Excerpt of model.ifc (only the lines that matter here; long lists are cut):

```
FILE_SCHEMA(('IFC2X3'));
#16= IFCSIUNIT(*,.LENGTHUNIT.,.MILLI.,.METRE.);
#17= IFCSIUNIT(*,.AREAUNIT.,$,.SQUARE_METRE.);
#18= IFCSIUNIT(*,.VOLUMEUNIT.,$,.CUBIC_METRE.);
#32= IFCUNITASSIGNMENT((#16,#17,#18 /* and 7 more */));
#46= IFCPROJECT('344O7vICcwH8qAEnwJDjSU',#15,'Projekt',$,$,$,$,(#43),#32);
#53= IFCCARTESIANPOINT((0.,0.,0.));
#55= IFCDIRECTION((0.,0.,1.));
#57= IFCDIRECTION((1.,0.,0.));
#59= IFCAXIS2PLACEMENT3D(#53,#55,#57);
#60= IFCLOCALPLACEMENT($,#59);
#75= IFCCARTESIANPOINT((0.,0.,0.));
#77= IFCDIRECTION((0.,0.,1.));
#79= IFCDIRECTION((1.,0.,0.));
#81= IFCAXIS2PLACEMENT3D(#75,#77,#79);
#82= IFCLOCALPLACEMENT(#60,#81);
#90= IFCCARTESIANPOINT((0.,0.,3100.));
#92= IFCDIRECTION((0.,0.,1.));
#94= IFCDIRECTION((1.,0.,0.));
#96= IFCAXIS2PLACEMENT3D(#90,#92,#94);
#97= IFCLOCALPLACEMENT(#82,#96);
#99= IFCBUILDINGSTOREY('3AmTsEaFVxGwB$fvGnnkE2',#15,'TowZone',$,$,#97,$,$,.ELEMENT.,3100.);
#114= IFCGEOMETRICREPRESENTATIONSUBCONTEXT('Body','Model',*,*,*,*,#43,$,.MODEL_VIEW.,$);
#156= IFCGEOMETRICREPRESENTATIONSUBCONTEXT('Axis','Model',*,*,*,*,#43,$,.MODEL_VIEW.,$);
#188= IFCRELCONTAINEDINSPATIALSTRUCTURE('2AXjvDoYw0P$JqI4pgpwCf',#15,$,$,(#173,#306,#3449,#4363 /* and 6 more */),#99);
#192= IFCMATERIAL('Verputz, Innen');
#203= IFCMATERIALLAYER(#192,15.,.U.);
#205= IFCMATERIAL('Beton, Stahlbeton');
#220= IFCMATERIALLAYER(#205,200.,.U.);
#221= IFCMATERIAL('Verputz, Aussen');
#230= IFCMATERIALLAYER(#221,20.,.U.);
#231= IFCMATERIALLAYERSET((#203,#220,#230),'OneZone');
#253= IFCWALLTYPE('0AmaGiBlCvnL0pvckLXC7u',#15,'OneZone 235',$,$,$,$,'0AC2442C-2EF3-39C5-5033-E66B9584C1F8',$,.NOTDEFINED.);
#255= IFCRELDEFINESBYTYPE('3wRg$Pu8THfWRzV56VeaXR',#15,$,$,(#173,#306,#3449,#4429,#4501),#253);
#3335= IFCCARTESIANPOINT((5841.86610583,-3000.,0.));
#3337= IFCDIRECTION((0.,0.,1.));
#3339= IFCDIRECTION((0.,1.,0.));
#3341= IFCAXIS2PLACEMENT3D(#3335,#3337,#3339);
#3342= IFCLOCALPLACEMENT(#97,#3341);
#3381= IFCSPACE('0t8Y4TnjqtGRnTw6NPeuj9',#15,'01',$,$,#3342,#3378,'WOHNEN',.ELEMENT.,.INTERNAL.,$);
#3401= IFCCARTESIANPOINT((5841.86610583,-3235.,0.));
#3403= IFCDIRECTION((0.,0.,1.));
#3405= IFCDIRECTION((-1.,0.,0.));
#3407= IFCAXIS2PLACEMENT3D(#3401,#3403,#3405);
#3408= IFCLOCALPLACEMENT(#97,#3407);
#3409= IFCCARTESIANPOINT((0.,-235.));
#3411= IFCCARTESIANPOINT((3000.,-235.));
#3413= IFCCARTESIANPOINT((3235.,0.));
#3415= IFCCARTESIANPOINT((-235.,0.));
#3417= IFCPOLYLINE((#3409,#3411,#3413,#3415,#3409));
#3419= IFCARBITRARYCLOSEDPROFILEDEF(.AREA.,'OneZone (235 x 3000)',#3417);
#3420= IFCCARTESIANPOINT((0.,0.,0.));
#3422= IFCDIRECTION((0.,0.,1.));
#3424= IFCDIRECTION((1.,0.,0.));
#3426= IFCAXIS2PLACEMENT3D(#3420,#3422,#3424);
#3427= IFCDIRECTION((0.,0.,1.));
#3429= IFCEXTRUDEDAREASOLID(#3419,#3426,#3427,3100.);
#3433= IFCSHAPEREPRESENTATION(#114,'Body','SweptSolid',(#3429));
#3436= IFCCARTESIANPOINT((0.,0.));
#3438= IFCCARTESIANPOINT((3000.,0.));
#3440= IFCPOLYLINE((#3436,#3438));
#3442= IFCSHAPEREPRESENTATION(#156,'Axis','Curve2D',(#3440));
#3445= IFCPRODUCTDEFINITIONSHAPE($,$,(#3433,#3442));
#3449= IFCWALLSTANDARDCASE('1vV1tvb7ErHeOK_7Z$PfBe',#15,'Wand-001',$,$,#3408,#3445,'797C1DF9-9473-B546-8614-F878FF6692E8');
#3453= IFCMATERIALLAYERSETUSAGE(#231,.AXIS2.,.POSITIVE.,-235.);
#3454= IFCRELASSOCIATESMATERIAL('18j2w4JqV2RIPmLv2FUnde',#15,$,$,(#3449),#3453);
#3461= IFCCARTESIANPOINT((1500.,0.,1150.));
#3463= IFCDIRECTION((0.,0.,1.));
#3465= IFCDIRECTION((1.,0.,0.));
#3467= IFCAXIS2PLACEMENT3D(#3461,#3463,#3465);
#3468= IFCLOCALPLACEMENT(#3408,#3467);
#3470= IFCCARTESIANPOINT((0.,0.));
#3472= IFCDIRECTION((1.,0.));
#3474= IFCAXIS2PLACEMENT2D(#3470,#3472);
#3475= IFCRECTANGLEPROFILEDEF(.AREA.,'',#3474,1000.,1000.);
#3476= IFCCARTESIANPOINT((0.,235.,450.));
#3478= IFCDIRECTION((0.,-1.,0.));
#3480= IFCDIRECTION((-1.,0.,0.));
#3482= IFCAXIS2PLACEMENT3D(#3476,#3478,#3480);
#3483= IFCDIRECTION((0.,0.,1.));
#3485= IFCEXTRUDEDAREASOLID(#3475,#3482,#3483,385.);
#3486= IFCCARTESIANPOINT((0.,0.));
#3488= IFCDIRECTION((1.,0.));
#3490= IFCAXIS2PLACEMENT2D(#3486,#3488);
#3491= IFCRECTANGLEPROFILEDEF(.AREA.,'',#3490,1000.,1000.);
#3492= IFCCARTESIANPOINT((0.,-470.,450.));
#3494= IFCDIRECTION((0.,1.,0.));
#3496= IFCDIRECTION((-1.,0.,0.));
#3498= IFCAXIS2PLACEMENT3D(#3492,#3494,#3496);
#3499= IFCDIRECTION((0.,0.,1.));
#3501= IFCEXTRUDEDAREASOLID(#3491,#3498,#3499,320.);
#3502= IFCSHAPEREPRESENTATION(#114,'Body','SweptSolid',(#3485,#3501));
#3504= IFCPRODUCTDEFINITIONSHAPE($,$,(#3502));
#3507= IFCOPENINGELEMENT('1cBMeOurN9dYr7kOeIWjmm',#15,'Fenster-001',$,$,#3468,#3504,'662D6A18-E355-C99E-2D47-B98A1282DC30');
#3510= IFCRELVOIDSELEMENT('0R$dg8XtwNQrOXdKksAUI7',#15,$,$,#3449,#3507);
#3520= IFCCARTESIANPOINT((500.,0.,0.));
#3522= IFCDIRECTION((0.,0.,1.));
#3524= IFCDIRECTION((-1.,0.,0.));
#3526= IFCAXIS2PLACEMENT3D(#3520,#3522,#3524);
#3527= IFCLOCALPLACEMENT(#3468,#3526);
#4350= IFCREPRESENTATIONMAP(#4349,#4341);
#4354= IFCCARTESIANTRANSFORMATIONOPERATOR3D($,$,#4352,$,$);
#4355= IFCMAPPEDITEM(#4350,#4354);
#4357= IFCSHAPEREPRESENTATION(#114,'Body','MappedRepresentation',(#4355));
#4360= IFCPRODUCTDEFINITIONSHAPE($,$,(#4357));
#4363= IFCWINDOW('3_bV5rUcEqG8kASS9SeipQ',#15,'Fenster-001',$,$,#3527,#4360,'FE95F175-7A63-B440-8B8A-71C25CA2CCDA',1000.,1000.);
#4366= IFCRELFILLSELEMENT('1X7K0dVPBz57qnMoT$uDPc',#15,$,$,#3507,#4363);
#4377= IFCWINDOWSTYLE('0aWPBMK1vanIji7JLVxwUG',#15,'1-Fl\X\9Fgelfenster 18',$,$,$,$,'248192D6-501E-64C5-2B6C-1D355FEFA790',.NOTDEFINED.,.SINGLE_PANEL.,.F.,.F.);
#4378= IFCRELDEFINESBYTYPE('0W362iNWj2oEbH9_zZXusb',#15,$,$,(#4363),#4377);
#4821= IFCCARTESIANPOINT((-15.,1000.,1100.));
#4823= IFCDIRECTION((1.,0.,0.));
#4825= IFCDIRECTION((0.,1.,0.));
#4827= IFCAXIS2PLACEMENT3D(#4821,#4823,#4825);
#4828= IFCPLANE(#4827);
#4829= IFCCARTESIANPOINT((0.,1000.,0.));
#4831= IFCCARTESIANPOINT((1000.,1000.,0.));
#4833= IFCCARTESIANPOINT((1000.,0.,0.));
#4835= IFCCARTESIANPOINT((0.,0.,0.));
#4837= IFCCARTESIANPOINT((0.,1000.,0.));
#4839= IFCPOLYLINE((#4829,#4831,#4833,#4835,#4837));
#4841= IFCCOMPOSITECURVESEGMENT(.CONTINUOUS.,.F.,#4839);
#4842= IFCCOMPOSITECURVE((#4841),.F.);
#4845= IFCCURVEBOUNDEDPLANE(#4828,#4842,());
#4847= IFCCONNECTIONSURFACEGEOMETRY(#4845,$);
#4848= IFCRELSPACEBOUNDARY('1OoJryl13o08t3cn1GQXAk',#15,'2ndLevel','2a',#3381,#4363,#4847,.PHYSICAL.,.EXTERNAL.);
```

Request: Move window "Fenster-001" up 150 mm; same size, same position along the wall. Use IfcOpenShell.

```python
import numpy as np
import ifcopenshell
import ifcopenshell.api.geometry
import ifcopenshell.util.placement
import ifcopenshell.util.unit

model = ifcopenshell.open("model.ifc")
unit_scale = ifcopenshell.util.unit.calculate_unit_scale(model)

window = model.by_id(4363)
opening = window.FillsVoids[0].RelatingOpeningElement
dz = 150.0

shift = np.array([0.0, 0.0, dz])
# The window is placed relative to its opening, so it follows when the opening moves.
matrix = ifcopenshell.util.placement.get_local_placement(opening.ObjectPlacement)
matrix[:3, 3] += shift
ifcopenshell.api.geometry.edit_object_placement(
    model, product=opening, matrix=matrix, is_si=False, should_transform_children=True
)

# Space boundary surfaces are stored in each space's coordinates; move them too.
for rel in window.ProvidesBoundaries:
    if not rel.ConnectionGeometry:
        continue
    surface = rel.ConnectionGeometry.SurfaceOnRelatingElement.BasisSurface
    space_matrix = ifcopenshell.util.placement.get_local_placement(rel.RelatingSpace.ObjectPlacement)
    point = np.array(surface.Position.Location.Coordinates) + space_matrix[:3, :3].T @ shift
    surface.Position = model.createIfcAxis2Placement3D(
        model.createIfcCartesianPoint(point.tolist()), surface.Position.Axis, surface.Position.RefDirection
    )

print(f"moved by {dz * unit_scale:+.3f} m")

model.write("model_v2.ifc")
```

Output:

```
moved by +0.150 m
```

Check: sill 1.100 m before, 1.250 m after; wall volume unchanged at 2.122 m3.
